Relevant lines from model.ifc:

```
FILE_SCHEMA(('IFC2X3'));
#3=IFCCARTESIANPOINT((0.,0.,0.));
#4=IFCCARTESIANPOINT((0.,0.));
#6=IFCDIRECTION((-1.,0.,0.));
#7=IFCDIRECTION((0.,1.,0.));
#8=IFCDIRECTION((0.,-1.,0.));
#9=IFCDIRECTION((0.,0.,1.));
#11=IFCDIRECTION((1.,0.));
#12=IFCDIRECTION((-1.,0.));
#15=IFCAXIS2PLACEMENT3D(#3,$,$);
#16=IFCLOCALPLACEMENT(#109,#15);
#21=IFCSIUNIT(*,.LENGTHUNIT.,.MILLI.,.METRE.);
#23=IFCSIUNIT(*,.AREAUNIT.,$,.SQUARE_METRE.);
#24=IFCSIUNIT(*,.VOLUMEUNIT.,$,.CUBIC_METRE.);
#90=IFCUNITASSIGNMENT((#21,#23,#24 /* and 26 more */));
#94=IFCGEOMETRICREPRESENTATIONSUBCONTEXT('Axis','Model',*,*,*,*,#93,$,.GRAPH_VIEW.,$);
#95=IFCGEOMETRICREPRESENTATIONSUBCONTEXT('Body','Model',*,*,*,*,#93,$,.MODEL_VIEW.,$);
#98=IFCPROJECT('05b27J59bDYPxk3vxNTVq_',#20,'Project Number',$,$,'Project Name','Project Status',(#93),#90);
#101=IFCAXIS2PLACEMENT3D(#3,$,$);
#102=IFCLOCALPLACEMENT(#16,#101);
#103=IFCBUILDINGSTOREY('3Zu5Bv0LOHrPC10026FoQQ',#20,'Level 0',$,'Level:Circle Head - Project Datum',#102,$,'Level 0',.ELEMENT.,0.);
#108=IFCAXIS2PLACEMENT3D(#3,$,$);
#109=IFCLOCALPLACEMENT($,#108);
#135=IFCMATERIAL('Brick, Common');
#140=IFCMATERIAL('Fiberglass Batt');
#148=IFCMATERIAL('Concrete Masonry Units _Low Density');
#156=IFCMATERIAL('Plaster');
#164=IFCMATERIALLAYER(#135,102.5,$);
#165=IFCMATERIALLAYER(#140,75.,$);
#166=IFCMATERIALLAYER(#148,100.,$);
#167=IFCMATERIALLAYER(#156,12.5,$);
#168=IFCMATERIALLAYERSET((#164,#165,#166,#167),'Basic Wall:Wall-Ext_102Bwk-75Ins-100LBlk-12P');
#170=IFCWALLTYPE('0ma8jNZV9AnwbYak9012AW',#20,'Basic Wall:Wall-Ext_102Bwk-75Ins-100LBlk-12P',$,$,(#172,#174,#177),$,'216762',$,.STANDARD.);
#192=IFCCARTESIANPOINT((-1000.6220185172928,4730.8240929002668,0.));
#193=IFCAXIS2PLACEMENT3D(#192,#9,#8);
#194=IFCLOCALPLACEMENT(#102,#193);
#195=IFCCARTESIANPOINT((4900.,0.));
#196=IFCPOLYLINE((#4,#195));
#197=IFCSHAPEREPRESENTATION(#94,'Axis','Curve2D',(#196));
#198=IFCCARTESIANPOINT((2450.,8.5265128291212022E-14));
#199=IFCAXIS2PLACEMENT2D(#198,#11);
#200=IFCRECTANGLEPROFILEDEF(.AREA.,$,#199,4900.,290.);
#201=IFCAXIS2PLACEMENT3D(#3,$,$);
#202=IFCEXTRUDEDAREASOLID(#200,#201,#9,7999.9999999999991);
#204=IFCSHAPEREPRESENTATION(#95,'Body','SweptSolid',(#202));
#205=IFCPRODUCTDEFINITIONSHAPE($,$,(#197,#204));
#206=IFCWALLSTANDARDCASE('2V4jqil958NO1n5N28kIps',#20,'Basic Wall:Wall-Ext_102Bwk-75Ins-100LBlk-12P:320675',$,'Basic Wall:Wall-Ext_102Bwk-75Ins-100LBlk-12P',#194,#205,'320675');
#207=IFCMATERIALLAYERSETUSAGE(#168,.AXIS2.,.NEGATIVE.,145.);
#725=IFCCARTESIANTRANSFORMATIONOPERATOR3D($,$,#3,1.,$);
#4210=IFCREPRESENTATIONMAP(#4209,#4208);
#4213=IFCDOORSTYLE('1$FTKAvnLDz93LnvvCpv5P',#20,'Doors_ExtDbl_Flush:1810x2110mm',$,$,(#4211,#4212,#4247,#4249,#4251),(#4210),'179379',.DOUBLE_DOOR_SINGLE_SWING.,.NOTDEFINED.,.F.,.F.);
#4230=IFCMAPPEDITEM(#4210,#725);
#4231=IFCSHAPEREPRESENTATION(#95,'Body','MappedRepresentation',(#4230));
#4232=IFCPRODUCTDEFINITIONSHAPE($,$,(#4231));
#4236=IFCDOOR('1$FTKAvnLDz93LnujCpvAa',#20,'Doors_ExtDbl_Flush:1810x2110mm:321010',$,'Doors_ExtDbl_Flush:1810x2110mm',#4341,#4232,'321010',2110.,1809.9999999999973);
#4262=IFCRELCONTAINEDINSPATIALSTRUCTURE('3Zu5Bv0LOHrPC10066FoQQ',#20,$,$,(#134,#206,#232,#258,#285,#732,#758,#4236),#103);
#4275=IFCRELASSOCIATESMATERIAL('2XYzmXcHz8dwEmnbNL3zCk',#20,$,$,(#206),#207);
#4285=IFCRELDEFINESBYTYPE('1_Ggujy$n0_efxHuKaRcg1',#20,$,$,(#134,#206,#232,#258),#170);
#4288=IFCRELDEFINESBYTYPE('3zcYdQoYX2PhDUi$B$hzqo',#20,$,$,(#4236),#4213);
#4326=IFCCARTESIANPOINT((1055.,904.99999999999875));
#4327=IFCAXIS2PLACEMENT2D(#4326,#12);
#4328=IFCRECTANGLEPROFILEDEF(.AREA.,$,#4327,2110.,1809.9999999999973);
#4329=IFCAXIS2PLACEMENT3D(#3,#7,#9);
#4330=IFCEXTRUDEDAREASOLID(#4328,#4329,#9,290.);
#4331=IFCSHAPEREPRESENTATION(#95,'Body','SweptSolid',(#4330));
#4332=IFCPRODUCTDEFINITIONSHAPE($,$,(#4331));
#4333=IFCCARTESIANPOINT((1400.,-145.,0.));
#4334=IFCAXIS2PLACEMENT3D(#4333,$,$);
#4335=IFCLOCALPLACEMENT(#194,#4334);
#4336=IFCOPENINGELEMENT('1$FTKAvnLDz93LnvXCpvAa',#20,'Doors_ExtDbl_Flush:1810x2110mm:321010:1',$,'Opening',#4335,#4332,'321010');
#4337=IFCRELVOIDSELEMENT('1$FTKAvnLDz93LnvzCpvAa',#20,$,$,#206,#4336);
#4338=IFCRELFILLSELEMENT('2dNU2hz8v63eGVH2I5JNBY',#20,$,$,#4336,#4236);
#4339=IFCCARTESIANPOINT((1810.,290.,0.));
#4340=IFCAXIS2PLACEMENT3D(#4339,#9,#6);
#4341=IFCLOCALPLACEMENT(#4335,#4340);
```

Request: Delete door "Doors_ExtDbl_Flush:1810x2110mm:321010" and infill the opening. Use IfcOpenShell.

```python
import ifcopenshell
import ifcopenshell.api.feature
import ifcopenshell.api.root
import ifcopenshell.geom
import ifcopenshell.util.shape

model = ifcopenshell.open("model.ifc")
settings = ifcopenshell.geom.settings()


def volume(element):
    """Net volume in cubic metres, openings subtracted."""
    shape = ifcopenshell.geom.create_shape(settings, element)
    return ifcopenshell.util.shape.get_volume(shape.geometry)


door = model.by_guid("1$FTKAvnLDz93LnujCpvAa")
opening = door.FillsVoids[0].RelatingOpeningElement
wall = opening.VoidsElements[0].RelatingBuildingElement
before = volume(wall)

ifcopenshell.api.root.remove_product(model, product=door)
ifcopenshell.api.feature.remove_feature(model, feature=opening)

after = volume(wall)

print(f"wall volume {before:.3f} -> {after:.3f} m3")

model.write("model_updated.ifc")
```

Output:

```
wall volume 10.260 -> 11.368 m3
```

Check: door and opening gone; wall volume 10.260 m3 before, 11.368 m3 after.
